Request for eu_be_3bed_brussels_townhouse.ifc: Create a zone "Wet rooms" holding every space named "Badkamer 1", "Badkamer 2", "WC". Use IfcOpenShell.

First a look at what the model holds.

```python
import ifcopenshell

model = ifcopenshell.open("eu_be_3bed_brussels_townhouse.ifc")
print(model.schema)
seen = {}
for space in model.by_type("IfcSpace"):
    seen[space.LongName] = seen.get(space.LongName, 0) + 1
for name, count in sorted(seen.items(), key=str):
    print(count, "x", name)
print("zones:", [z.Name for z in model.by_type("IfcZone")][:20])
```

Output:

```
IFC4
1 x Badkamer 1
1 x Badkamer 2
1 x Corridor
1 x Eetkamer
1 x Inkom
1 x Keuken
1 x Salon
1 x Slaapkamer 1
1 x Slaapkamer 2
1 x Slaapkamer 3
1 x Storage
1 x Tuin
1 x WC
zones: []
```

```python
import ifcopenshell
import ifcopenshell.api.group
import ifcopenshell.api.root

model = ifcopenshell.open("eu_be_3bed_brussels_townhouse.ifc")

names = {"Badkamer 1", "Badkamer 2", "WC"}
spaces = [s for s in model.by_type("IfcSpace") if s.LongName in names]

zone = ifcopenshell.api.root.create_entity(model, ifc_class="IfcZone", name="Wet rooms")
ifcopenshell.api.group.assign_group(model, products=spaces, group=zone)
print(len(spaces), "spaces in", zone.Name)

model.write("eu_be_3bed_brussels_townhouse_rev.ifc")
```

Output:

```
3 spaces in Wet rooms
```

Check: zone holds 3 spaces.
